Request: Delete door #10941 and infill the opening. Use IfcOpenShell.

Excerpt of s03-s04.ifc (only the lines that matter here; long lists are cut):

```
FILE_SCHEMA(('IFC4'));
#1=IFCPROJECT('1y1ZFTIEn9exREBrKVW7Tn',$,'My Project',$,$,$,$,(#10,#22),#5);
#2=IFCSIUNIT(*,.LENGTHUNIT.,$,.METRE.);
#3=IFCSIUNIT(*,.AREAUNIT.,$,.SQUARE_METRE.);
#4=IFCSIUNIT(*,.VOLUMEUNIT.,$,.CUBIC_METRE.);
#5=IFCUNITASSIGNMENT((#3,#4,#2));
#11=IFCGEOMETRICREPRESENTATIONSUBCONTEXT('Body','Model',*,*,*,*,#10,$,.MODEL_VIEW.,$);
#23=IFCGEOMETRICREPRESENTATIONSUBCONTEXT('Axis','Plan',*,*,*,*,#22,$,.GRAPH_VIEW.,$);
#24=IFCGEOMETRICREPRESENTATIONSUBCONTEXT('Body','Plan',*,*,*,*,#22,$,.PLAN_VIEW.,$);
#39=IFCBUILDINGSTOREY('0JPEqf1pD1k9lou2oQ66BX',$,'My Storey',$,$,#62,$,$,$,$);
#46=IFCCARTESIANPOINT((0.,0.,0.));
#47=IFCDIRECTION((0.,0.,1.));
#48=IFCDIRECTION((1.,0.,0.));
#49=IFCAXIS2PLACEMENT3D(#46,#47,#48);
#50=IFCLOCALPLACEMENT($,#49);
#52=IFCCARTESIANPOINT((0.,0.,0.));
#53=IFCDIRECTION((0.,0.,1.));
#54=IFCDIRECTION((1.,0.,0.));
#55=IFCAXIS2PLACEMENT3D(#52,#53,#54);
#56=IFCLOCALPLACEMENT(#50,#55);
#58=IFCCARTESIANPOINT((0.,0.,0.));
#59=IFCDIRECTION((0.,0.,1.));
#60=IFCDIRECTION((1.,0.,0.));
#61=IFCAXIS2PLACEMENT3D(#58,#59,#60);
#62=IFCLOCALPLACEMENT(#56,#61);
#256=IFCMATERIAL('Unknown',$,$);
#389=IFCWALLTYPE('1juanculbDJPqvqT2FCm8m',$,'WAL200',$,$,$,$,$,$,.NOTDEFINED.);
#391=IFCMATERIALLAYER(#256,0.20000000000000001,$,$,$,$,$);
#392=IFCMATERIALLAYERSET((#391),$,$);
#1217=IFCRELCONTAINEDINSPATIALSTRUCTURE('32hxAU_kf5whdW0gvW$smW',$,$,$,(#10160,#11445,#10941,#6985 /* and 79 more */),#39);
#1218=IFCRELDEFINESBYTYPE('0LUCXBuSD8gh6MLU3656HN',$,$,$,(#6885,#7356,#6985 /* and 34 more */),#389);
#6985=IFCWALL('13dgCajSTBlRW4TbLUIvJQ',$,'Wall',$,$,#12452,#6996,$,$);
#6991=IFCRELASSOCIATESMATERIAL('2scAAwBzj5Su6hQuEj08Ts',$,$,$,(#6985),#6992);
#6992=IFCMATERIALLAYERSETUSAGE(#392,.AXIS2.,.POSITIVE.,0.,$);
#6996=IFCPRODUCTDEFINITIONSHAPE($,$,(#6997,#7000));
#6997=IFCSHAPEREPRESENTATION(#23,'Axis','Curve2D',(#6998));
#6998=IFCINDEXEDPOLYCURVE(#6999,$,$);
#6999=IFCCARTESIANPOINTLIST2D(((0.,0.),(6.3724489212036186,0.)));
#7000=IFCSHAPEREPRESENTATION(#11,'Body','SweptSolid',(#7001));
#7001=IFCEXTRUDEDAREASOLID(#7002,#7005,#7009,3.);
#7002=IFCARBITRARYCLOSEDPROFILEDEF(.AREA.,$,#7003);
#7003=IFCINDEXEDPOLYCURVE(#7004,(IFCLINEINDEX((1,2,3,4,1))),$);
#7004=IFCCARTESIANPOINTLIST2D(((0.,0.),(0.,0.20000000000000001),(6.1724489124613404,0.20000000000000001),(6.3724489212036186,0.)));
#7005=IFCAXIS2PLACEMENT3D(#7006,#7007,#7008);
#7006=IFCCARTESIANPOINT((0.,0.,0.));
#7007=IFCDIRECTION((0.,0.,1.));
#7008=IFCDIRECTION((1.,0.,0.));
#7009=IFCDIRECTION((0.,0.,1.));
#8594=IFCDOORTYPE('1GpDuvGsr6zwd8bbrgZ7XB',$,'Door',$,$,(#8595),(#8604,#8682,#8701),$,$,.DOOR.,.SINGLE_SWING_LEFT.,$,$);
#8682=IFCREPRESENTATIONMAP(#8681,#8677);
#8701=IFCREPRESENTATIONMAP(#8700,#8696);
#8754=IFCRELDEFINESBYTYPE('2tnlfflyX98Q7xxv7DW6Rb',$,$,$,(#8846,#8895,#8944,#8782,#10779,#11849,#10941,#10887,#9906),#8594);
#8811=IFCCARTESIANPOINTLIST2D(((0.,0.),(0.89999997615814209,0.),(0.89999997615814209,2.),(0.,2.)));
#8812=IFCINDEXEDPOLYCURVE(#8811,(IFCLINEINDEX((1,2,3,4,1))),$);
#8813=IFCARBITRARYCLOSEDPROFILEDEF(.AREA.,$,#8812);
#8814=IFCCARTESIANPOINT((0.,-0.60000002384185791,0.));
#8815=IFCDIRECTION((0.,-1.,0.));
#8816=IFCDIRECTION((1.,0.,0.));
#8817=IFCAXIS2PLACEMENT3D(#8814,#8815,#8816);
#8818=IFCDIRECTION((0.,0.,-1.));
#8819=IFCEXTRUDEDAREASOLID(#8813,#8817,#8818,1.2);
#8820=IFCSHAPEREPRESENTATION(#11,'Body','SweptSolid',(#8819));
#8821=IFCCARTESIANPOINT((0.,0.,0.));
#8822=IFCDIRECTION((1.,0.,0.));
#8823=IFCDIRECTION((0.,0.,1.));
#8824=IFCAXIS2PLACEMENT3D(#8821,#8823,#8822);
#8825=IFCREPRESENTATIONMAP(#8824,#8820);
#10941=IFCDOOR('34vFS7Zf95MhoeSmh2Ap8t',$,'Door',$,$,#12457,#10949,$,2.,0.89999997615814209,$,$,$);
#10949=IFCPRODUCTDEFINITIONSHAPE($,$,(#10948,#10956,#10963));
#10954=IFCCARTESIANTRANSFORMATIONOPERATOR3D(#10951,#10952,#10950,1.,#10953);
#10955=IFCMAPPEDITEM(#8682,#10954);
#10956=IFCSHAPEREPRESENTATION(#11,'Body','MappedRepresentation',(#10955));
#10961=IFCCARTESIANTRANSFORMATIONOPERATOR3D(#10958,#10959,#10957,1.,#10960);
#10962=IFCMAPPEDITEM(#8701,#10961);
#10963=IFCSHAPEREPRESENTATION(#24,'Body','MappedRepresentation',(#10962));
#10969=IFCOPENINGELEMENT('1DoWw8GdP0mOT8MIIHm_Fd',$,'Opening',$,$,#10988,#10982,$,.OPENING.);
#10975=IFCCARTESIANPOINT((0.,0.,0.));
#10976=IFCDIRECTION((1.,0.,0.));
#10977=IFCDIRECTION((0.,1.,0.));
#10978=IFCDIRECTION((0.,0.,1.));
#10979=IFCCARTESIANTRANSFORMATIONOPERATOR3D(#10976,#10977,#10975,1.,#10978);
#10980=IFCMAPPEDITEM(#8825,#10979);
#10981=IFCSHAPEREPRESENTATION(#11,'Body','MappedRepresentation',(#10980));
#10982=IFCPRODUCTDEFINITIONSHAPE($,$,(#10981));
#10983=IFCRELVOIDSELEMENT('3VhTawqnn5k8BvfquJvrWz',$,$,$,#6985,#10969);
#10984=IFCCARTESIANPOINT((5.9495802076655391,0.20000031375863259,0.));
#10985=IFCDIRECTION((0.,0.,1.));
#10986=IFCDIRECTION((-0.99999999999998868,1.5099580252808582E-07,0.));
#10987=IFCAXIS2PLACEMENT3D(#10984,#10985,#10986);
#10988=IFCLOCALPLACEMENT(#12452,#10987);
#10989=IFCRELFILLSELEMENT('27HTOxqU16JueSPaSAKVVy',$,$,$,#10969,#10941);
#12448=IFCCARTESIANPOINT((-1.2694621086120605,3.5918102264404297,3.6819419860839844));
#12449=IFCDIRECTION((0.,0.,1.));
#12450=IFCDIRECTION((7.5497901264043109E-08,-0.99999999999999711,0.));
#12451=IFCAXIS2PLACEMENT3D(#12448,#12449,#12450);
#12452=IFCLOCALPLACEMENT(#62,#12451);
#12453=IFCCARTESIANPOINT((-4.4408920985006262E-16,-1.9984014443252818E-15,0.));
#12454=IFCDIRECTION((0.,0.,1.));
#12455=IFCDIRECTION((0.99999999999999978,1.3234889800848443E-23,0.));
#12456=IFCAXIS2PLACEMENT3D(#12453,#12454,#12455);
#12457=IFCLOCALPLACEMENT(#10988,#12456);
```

```python
import ifcopenshell
import ifcopenshell.api.feature
import ifcopenshell.api.root
import ifcopenshell.geom
import ifcopenshell.util.shape

model = ifcopenshell.open("s03-s04.ifc")
settings = ifcopenshell.geom.settings()


def volume(element):
    """Net volume in cubic metres, openings subtracted."""
    shape = ifcopenshell.geom.create_shape(settings, element)
    return ifcopenshell.util.shape.get_volume(shape.geometry)


door = model.by_guid("34vFS7Zf95MhoeSmh2Ap8t")
opening = door.FillsVoids[0].RelatingOpeningElement
wall = opening.VoidsElements[0].RelatingBuildingElement
before = volume(wall)

ifcopenshell.api.root.remove_product(model, product=door)
ifcopenshell.api.feature.remove_feature(model, feature=opening)

after = volume(wall)

print(f"wall volume {before:.3f} -> {after:.3f} m3")

model.write("s03-s04_updated.ifc")
```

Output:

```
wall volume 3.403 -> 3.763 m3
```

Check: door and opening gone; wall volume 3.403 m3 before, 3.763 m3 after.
